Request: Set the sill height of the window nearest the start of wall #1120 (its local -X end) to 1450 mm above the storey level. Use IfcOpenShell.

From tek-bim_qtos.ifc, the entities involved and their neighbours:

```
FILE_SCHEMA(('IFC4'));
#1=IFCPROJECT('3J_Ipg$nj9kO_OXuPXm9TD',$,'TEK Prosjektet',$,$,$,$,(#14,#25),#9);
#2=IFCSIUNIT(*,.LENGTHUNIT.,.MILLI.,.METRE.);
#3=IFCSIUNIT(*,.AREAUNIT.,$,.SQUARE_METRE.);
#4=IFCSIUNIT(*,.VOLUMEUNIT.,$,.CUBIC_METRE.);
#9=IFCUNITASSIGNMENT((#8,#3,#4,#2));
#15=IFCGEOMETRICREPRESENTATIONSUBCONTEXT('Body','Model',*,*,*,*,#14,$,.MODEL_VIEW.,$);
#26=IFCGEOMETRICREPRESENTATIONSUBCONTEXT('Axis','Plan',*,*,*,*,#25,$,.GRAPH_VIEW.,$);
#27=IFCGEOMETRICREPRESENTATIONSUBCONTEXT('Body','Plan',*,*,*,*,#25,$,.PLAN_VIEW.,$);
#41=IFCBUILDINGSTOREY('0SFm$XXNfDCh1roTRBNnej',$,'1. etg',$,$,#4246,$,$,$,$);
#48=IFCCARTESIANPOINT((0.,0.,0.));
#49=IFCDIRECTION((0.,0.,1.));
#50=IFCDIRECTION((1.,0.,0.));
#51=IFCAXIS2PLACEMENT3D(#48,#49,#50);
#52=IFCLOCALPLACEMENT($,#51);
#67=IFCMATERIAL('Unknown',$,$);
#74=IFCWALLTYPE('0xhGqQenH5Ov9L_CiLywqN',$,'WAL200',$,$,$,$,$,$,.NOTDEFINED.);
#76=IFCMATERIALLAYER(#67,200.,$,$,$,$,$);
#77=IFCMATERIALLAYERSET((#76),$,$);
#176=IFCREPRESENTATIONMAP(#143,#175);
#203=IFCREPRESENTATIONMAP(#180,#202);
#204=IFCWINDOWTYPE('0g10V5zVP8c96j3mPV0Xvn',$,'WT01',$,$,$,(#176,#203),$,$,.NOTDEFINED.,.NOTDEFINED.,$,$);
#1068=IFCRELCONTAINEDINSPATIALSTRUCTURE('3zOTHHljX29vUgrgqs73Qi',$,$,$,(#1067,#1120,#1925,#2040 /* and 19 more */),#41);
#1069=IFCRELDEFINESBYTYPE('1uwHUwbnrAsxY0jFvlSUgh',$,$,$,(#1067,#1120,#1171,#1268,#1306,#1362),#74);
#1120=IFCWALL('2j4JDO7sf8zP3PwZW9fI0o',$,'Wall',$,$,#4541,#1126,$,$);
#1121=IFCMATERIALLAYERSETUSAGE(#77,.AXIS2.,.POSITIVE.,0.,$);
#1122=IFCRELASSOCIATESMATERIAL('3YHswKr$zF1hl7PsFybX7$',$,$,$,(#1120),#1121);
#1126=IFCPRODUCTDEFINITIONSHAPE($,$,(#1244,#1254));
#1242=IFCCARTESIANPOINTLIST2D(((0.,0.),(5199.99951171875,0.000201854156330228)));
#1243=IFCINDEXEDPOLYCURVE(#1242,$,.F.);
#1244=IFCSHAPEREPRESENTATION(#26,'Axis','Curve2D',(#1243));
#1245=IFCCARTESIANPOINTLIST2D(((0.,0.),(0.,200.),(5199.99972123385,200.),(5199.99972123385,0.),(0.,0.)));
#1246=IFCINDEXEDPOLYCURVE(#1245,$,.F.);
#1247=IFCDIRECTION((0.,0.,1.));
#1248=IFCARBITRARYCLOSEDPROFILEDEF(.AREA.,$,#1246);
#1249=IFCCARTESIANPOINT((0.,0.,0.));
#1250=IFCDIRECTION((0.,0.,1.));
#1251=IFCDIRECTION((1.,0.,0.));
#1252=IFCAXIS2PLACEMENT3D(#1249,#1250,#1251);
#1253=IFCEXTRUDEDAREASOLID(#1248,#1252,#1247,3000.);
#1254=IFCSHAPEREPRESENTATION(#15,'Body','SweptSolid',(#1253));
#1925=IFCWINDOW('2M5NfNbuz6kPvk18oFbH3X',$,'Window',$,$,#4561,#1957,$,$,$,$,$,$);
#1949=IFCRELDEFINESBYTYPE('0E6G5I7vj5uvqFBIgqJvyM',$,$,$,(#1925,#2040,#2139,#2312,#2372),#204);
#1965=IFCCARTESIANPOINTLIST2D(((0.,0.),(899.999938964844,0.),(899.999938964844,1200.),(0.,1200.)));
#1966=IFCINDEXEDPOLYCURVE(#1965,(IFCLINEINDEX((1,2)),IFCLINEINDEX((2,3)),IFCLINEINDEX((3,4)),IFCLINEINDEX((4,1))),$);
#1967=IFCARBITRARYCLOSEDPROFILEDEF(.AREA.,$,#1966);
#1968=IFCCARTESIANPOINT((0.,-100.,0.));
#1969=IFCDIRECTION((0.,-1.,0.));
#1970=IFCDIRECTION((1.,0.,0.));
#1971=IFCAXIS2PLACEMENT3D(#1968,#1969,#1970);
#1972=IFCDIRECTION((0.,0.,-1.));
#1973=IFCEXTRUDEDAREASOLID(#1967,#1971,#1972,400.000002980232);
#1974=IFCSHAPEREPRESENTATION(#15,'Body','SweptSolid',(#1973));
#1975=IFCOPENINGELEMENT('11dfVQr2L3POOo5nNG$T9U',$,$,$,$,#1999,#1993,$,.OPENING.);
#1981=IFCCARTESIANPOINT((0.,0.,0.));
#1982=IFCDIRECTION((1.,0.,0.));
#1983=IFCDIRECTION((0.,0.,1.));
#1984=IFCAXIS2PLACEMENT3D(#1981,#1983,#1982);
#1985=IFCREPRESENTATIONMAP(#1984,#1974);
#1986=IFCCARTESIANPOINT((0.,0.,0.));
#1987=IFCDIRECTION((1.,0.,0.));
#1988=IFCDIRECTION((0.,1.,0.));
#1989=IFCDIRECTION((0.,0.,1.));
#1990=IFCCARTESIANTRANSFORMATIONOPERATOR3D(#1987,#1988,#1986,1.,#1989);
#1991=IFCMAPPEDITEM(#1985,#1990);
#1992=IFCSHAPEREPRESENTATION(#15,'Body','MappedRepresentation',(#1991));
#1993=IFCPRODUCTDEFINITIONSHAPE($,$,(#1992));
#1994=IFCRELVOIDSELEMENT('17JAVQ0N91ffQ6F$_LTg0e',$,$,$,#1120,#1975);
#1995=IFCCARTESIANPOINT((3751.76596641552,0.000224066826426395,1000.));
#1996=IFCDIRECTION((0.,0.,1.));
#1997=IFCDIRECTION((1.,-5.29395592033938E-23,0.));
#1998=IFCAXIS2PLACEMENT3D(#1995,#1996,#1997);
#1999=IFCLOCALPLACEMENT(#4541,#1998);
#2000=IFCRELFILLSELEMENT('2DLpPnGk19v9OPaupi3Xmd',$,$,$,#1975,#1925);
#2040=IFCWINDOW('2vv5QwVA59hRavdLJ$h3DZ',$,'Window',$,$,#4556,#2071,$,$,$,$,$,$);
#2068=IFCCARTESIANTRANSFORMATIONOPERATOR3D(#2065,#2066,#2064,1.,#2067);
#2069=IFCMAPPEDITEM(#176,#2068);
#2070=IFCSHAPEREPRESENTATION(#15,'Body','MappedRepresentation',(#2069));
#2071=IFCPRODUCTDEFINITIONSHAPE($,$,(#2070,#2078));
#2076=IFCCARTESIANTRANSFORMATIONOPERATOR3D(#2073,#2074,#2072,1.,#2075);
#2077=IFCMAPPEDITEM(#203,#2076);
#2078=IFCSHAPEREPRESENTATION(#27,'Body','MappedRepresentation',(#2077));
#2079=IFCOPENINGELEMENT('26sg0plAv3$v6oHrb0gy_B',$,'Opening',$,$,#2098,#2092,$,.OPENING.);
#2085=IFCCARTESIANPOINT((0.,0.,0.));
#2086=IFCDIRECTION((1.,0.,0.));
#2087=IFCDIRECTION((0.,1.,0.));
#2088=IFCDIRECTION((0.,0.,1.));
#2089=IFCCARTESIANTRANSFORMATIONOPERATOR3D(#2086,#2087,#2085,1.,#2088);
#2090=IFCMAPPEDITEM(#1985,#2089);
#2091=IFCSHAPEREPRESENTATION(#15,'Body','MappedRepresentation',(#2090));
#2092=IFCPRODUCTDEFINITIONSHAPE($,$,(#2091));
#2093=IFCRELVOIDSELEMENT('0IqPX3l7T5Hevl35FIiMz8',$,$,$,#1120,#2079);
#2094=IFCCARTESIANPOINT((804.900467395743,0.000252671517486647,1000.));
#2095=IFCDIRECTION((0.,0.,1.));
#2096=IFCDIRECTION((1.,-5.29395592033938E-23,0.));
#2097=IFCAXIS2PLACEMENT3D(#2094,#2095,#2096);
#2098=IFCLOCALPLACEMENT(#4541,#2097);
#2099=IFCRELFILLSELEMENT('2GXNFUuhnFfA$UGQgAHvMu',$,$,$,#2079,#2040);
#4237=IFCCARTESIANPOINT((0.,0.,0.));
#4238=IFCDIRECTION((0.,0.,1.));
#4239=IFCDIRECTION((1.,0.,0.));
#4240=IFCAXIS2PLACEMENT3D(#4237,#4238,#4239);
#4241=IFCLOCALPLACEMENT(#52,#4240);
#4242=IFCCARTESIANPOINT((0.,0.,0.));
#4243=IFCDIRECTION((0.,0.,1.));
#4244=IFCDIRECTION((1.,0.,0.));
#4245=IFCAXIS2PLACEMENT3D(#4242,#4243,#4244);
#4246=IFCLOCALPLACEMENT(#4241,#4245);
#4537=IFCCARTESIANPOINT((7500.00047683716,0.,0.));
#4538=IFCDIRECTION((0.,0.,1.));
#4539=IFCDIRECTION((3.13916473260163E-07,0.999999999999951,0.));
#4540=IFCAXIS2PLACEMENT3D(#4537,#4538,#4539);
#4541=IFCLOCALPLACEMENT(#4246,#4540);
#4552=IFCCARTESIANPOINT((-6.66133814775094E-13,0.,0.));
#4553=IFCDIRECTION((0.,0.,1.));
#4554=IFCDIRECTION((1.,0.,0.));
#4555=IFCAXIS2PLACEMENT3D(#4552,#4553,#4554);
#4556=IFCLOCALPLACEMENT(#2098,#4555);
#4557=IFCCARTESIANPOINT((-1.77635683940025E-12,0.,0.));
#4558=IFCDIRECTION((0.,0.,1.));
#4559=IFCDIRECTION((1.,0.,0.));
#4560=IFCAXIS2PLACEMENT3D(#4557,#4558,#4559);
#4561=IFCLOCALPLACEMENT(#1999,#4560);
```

```python
import numpy as np
import ifcopenshell
import ifcopenshell.api.geometry
import ifcopenshell.geom
import ifcopenshell.util.element
import ifcopenshell.util.placement
import ifcopenshell.util.shape
import ifcopenshell.util.unit

model = ifcopenshell.open("tek-bim_qtos.ifc")
unit_scale = ifcopenshell.util.unit.calculate_unit_scale(model)

window = model.by_id(2040)
opening = window.FillsVoids[0].RelatingOpeningElement
storey = ifcopenshell.util.element.get_container(window, ifc_class="IfcBuildingStorey")
level = ifcopenshell.util.placement.get_local_placement(storey.ObjectPlacement)[2, 3]

# The opening's origin need not be at the sill, so measure its lowest point.
shape = ifcopenshell.geom.create_shape(ifcopenshell.geom.settings(), opening)
bottom = ifcopenshell.util.shape.get_shape_bottom_elevation(shape, shape.geometry) / unit_scale
dz = level + 1.45 / unit_scale - bottom

shift = np.array([0.0, 0.0, dz])
# The window is placed relative to its opening, so it follows when the opening moves.
matrix = ifcopenshell.util.placement.get_local_placement(opening.ObjectPlacement)
matrix[:3, 3] += shift
ifcopenshell.api.geometry.edit_object_placement(
    model, product=opening, matrix=matrix, is_si=False, should_transform_children=True
)

print(f"moved by {dz * unit_scale:+.3f} m")

model.write("tek-bim_qtos-out.ifc")
```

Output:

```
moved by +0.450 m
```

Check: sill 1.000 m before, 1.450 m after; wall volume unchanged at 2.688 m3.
